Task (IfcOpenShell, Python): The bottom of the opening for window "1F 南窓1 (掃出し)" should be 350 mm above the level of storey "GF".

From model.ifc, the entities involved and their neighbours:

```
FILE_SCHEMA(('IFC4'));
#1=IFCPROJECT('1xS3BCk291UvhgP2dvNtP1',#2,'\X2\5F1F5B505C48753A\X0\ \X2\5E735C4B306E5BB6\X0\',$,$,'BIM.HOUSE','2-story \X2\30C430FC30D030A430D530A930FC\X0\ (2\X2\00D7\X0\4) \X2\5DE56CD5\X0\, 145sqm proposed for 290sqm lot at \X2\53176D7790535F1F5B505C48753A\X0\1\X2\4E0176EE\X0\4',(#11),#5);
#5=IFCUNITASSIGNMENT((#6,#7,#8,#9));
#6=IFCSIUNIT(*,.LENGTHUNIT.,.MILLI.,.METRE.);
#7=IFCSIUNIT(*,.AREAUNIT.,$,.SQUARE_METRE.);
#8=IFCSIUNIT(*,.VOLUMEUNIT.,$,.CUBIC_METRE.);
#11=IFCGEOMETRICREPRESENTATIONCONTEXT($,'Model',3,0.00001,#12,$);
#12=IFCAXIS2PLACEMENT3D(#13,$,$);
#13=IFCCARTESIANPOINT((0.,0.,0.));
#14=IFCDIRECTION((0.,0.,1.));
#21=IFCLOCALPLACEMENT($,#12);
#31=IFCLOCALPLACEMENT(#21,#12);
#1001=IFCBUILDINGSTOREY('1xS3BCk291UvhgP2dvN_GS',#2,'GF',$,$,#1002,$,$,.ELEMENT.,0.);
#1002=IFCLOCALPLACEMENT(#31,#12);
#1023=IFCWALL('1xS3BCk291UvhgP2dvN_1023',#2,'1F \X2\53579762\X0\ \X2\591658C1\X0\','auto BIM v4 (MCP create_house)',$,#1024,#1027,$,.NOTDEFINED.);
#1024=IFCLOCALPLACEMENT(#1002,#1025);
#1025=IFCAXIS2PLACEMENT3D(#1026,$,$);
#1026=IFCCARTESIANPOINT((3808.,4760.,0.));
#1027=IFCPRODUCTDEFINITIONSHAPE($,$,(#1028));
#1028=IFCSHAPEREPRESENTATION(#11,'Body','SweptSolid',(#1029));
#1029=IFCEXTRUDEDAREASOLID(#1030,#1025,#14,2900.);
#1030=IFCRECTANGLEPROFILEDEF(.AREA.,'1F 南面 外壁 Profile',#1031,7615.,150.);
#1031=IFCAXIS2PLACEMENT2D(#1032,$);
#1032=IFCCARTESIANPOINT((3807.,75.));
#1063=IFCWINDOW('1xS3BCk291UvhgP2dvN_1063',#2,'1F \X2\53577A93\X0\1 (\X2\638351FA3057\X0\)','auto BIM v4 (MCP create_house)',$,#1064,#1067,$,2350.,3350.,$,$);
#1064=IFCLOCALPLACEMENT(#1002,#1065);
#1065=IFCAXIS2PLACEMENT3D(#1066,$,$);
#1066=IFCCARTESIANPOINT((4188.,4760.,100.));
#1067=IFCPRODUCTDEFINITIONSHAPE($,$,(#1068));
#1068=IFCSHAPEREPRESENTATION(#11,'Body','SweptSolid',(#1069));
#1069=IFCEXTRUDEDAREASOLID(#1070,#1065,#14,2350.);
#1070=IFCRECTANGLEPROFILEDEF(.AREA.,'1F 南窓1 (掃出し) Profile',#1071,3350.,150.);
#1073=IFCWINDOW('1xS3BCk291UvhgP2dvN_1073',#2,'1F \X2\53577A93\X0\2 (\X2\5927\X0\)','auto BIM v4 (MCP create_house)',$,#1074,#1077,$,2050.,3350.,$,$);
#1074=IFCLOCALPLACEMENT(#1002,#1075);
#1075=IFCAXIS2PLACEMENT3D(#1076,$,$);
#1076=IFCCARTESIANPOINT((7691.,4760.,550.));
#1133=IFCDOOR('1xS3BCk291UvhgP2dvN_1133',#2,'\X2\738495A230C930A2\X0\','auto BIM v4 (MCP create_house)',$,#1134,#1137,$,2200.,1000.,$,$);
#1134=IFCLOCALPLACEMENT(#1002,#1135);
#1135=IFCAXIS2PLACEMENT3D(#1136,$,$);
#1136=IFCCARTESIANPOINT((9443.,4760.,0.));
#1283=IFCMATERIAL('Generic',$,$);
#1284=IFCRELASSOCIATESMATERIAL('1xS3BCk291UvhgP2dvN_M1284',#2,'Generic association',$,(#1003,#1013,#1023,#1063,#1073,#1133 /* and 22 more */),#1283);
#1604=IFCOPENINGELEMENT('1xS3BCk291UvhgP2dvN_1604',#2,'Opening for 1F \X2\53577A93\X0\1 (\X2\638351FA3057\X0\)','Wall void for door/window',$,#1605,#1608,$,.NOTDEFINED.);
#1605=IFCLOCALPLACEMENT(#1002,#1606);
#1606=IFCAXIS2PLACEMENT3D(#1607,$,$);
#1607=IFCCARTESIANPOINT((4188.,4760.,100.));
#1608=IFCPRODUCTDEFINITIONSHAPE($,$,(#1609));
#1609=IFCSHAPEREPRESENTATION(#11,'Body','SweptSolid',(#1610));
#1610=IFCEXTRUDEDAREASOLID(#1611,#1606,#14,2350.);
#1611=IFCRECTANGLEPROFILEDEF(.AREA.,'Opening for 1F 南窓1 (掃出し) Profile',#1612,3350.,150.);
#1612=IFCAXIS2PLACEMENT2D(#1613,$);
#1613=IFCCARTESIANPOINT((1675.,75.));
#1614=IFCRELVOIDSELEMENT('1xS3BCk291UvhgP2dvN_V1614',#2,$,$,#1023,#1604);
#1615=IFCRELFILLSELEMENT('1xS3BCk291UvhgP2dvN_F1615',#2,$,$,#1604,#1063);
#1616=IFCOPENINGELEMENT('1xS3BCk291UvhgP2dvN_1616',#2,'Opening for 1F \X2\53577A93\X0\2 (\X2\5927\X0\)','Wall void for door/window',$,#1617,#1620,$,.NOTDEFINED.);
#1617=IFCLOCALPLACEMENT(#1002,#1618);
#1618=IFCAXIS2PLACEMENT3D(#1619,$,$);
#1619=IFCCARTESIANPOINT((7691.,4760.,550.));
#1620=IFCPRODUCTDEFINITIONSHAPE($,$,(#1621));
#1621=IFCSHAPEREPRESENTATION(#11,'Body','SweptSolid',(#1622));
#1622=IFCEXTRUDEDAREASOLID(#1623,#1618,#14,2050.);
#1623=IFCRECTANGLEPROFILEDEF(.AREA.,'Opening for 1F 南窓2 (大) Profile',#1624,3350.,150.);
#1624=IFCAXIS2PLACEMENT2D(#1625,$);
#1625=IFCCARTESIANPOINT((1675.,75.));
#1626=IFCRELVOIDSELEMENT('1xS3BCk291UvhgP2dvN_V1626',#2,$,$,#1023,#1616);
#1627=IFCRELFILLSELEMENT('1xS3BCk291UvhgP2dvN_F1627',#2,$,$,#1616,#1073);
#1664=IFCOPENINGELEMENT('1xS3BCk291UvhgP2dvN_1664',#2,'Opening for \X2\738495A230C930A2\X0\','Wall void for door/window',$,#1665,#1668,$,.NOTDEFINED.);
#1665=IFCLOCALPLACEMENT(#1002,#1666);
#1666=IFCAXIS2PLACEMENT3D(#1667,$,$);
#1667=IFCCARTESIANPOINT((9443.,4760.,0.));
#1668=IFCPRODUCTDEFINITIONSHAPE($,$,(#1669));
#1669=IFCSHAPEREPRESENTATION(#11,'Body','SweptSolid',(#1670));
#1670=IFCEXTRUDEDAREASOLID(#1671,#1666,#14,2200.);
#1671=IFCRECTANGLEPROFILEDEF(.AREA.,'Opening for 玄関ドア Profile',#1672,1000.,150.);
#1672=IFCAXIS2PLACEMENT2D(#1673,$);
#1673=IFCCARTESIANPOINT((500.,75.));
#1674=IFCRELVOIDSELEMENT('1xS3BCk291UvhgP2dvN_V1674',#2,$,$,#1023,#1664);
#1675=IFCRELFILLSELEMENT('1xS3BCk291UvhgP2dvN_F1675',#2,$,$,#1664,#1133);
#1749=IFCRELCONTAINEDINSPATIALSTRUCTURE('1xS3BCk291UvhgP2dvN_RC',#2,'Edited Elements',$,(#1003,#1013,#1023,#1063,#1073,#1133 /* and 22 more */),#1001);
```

```python
import numpy as np
import ifcopenshell
import ifcopenshell.api.geometry
import ifcopenshell.geom
import ifcopenshell.util.element
import ifcopenshell.util.placement
import ifcopenshell.util.shape
import ifcopenshell.util.unit

model = ifcopenshell.open("model.ifc")
unit_scale = ifcopenshell.util.unit.calculate_unit_scale(model)

window = model.by_guid("1xS3BCk291UvhgP2dvN_1063")
opening = window.FillsVoids[0].RelatingOpeningElement
storey = ifcopenshell.util.element.get_container(window, ifc_class="IfcBuildingStorey")
level = ifcopenshell.util.placement.get_local_placement(storey.ObjectPlacement)[2, 3]

# The opening's origin need not be at the sill, so measure its lowest point.
shape = ifcopenshell.geom.create_shape(ifcopenshell.geom.settings(), opening)
bottom = ifcopenshell.util.shape.get_shape_bottom_elevation(shape, shape.geometry) / unit_scale
dz = level + 0.35 / unit_scale - bottom

shift = np.array([0.0, 0.0, dz])
# The window is not placed relative to its opening, so move both.
for product in (opening, window):
    matrix = ifcopenshell.util.placement.get_local_placement(product.ObjectPlacement)
    matrix[:3, 3] += shift
    ifcopenshell.api.geometry.edit_object_placement(model, product=product, matrix=matrix, is_si=False)

print(f"moved by {dz * unit_scale:+.3f} m")

model.write("model-out.ifc")
```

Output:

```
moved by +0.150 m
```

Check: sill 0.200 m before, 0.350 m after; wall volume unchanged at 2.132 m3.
